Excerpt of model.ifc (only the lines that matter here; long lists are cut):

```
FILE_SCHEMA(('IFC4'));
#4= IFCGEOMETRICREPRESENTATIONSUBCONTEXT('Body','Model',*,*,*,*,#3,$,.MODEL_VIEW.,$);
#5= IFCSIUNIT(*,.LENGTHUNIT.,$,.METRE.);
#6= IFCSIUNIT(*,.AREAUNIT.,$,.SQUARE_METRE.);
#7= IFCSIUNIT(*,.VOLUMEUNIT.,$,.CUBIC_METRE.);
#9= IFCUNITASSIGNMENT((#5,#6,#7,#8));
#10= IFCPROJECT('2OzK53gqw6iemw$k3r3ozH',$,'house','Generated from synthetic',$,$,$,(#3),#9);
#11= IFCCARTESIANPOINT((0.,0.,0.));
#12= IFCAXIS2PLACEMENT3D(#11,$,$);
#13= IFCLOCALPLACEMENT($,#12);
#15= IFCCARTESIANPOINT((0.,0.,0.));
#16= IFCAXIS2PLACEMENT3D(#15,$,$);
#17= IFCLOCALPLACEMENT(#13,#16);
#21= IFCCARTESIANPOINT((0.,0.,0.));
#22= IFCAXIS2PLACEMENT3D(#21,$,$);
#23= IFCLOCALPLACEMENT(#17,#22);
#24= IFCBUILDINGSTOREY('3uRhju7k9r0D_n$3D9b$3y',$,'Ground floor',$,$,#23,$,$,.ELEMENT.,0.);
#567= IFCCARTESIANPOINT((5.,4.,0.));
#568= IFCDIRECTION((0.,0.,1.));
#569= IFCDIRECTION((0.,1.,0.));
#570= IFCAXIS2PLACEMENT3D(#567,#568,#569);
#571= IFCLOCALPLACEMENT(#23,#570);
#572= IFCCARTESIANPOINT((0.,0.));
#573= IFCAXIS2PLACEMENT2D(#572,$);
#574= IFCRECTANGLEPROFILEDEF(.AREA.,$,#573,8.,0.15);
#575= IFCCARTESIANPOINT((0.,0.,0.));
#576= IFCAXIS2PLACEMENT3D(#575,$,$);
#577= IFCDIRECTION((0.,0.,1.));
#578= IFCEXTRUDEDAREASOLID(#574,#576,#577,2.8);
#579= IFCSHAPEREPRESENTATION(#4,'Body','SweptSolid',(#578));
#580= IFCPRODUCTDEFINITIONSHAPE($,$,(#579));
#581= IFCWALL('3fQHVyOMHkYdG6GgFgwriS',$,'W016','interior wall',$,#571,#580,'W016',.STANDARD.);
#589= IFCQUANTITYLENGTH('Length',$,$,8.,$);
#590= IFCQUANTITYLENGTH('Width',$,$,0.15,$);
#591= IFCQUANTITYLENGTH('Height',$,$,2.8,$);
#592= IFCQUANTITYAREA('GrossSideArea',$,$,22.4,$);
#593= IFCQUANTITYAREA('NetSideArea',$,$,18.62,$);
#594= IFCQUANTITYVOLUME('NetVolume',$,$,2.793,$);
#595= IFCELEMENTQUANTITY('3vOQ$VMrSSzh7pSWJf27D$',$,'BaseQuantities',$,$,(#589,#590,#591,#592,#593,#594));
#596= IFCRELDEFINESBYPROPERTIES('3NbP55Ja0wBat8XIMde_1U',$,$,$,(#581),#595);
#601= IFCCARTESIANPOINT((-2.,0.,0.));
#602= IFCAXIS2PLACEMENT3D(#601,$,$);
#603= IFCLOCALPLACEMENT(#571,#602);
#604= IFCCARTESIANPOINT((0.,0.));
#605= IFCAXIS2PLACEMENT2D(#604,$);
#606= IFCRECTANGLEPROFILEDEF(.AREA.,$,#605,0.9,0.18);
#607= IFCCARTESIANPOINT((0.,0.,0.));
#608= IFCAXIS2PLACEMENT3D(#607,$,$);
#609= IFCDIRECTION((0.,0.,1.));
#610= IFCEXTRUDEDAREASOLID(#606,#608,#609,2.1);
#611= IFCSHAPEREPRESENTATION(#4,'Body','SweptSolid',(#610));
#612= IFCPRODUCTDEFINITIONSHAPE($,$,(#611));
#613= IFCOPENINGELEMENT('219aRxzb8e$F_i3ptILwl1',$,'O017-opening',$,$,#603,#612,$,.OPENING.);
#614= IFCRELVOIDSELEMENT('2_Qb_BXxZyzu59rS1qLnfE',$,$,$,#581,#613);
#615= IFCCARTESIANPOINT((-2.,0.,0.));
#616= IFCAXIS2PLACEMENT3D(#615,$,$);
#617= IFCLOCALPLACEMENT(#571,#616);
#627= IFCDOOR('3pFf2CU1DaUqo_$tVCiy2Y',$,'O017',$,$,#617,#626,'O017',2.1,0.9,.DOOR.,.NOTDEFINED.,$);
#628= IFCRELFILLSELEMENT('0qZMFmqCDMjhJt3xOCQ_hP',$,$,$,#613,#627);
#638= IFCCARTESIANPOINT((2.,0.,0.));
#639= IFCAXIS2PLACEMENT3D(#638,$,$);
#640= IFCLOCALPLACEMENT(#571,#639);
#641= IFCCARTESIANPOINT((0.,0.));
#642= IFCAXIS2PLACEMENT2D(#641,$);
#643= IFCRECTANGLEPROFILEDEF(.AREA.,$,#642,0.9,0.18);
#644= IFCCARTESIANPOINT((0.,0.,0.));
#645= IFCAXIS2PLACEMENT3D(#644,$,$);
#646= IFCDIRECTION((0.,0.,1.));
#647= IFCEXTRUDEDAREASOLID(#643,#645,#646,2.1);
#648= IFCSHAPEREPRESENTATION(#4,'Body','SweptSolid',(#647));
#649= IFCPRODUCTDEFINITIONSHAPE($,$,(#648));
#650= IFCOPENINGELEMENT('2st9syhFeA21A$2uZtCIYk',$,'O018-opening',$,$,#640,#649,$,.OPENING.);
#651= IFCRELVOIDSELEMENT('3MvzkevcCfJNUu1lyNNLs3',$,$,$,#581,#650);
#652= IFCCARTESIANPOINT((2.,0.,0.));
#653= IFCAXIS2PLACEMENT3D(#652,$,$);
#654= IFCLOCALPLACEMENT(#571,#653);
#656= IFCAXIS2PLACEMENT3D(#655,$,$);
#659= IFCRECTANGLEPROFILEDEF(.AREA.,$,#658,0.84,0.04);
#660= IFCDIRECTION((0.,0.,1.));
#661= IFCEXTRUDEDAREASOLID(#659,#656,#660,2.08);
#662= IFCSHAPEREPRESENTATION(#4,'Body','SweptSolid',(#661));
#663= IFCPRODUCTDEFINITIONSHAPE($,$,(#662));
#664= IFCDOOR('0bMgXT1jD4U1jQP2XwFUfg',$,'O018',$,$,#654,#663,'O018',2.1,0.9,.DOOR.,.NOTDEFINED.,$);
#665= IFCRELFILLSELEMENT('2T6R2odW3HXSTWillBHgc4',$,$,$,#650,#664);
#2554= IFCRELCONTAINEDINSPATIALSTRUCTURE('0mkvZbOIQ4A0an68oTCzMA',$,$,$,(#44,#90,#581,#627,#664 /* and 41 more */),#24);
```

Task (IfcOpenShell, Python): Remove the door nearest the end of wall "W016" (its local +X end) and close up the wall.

```python
import ifcopenshell
import ifcopenshell.api.feature
import ifcopenshell.api.pset
import ifcopenshell.api.root
import ifcopenshell.geom
import ifcopenshell.util.element
import ifcopenshell.util.shape
import ifcopenshell.util.unit

model = ifcopenshell.open("model.ifc")
area_scale = ifcopenshell.util.unit.calculate_unit_scale(model, "AREAUNIT")
volume_scale = ifcopenshell.util.unit.calculate_unit_scale(model, "VOLUMEUNIT")
settings = ifcopenshell.geom.settings()


def volume(element):
    """Net volume in cubic metres, openings subtracted."""
    shape = ifcopenshell.geom.create_shape(settings, element)
    return ifcopenshell.util.shape.get_volume(shape.geometry)


door = model.by_guid("0bMgXT1jD4U1jQP2XwFUfg")
opening = door.FillsVoids[0].RelatingOpeningElement
wall = opening.VoidsElements[0].RelatingBuildingElement
before = volume(wall)

ifcopenshell.api.root.remove_product(model, product=door)
ifcopenshell.api.feature.remove_feature(model, feature=opening)

after = volume(wall)
thickness = 0.15  # wall thickness in metres

# Update the wall's stored quantities.
qto = model.by_id(ifcopenshell.util.element.get_pset(wall, "BaseQuantities", should_inherit=False)["id"])
ifcopenshell.api.pset.edit_qto(model, qto=qto, properties={
    "NetSideArea": after / thickness / area_scale,
    "NetVolume": after / volume_scale,
})

print(f"wall volume {before:.3f} -> {after:.3f} m3")

model.write("model_v2.ifc")
```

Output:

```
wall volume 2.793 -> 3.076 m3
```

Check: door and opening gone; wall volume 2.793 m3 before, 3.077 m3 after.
